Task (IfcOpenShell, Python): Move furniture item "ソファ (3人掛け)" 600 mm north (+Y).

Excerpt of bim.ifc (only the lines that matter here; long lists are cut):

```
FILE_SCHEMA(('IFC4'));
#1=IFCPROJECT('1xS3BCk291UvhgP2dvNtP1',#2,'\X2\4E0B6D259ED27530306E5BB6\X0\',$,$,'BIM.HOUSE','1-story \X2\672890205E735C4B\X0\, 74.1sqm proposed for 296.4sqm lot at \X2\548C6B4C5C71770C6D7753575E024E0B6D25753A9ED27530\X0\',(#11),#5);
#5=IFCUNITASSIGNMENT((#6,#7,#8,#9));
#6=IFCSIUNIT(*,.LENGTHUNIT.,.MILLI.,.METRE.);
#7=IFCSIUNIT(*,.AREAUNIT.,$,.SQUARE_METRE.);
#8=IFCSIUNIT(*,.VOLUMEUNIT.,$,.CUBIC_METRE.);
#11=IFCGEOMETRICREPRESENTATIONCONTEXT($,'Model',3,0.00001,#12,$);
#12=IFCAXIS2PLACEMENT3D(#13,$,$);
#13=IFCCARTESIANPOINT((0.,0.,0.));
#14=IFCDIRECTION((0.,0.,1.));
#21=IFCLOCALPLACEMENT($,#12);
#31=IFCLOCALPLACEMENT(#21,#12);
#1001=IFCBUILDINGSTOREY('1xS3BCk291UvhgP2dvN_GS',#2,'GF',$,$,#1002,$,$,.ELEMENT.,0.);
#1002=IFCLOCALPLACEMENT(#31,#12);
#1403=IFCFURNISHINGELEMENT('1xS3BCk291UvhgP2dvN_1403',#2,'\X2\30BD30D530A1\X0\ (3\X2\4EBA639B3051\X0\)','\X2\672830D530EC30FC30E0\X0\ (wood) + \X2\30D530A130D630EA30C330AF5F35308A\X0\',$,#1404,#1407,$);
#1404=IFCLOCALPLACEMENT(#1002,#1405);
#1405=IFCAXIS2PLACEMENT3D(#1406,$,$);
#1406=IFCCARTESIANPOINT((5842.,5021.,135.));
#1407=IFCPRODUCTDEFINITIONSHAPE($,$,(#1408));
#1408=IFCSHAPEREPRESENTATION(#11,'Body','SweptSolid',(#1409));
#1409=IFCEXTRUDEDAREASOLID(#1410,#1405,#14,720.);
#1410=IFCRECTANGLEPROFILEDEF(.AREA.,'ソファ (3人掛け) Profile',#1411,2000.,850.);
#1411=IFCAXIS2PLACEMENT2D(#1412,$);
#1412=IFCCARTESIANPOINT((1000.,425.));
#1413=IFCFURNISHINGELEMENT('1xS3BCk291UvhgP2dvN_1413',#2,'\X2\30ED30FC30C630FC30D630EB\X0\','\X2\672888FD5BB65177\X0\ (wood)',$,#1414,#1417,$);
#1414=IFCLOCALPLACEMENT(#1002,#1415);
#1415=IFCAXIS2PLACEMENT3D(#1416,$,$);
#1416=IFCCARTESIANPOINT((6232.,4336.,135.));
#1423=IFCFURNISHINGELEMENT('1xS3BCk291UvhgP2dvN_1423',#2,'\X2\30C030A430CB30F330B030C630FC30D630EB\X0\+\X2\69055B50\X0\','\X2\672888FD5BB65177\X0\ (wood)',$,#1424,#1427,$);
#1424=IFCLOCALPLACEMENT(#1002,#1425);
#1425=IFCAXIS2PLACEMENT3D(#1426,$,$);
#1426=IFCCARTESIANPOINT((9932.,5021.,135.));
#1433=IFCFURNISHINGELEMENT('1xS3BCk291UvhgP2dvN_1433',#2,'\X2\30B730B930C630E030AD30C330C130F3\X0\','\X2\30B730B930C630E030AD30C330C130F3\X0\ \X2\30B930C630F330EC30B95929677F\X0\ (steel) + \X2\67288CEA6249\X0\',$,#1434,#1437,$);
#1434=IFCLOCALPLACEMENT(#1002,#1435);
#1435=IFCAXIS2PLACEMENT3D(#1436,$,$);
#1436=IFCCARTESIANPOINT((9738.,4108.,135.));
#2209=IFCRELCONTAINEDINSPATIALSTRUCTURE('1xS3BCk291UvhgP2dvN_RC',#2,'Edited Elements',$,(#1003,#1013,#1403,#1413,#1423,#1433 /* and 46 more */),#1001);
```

```python
import ifcopenshell
import ifcopenshell.api.geometry
import ifcopenshell.util.placement
import ifcopenshell.util.unit

model = ifcopenshell.open("bim.ifc")
unit_scale = ifcopenshell.util.unit.calculate_unit_scale(model)

item = model.by_guid("1xS3BCk291UvhgP2dvN_1403")
matrix = ifcopenshell.util.placement.get_local_placement(item.ObjectPlacement)
matrix[1, 3] += 0.6 / unit_scale
ifcopenshell.api.geometry.edit_object_placement(model, product=item, matrix=matrix, is_si=False)

print(ifcopenshell.util.placement.get_local_placement(item.ObjectPlacement).round(3) + 0.0)

model.write("bim-out.ifc")
```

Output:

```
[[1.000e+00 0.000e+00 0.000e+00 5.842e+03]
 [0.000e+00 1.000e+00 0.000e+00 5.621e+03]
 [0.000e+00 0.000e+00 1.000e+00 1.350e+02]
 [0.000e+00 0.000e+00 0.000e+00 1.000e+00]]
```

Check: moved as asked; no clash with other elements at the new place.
